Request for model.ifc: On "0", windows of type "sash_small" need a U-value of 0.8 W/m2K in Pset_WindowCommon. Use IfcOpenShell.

First a look at what the model holds.

```python
import ifcopenshell
import ifcopenshell.util.element

model = ifcopenshell.open("model.ifc")
print(model.schema)
storey = next(s for s in model.by_type("IfcBuildingStorey") if s.Name == "0")
windows = [e for e in ifcopenshell.util.element.get_decomposition(storey) if e.is_a("IfcWindow")]
seen = {}
for e in windows:
    element_type = ifcopenshell.util.element.get_type(e)
    key = (element_type.Name if element_type != e and element_type else None, ifcopenshell.util.element.get_pset(e, "Pset_WindowCommon", "ThermalTransmittance"))
    seen[key] = seen.get(key, 0) + 1
for (name, value), count in sorted(seen.items(), key=str):
    print(count, "x", name, "|", value)
```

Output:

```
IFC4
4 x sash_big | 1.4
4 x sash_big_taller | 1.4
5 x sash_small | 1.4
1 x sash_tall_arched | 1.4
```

```python
import ifcopenshell
import ifcopenshell.api.pset
import ifcopenshell.util.element

model = ifcopenshell.open("model.ifc")

storey = next(s for s in model.by_type("IfcBuildingStorey") if s.Name == "0")
windows = [e for e in ifcopenshell.util.element.get_decomposition(storey) if e.is_a("IfcWindow")]

count = 0
for e in windows:
    element_type = ifcopenshell.util.element.get_type(e)
    if element_type in (None, e) or element_type.Name != "sash_small":
        continue
    # add_pset returns the element's existing set when there is one.
    pset = ifcopenshell.api.pset.add_pset(model, product=e, name="Pset_WindowCommon")
    ifcopenshell.api.pset.edit_pset(model, pset=pset, properties={"ThermalTransmittance": 0.8})
    count += 1

print(count, "windows updated")

model.write("model_edited.ifc")
```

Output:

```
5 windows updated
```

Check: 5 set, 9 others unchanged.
